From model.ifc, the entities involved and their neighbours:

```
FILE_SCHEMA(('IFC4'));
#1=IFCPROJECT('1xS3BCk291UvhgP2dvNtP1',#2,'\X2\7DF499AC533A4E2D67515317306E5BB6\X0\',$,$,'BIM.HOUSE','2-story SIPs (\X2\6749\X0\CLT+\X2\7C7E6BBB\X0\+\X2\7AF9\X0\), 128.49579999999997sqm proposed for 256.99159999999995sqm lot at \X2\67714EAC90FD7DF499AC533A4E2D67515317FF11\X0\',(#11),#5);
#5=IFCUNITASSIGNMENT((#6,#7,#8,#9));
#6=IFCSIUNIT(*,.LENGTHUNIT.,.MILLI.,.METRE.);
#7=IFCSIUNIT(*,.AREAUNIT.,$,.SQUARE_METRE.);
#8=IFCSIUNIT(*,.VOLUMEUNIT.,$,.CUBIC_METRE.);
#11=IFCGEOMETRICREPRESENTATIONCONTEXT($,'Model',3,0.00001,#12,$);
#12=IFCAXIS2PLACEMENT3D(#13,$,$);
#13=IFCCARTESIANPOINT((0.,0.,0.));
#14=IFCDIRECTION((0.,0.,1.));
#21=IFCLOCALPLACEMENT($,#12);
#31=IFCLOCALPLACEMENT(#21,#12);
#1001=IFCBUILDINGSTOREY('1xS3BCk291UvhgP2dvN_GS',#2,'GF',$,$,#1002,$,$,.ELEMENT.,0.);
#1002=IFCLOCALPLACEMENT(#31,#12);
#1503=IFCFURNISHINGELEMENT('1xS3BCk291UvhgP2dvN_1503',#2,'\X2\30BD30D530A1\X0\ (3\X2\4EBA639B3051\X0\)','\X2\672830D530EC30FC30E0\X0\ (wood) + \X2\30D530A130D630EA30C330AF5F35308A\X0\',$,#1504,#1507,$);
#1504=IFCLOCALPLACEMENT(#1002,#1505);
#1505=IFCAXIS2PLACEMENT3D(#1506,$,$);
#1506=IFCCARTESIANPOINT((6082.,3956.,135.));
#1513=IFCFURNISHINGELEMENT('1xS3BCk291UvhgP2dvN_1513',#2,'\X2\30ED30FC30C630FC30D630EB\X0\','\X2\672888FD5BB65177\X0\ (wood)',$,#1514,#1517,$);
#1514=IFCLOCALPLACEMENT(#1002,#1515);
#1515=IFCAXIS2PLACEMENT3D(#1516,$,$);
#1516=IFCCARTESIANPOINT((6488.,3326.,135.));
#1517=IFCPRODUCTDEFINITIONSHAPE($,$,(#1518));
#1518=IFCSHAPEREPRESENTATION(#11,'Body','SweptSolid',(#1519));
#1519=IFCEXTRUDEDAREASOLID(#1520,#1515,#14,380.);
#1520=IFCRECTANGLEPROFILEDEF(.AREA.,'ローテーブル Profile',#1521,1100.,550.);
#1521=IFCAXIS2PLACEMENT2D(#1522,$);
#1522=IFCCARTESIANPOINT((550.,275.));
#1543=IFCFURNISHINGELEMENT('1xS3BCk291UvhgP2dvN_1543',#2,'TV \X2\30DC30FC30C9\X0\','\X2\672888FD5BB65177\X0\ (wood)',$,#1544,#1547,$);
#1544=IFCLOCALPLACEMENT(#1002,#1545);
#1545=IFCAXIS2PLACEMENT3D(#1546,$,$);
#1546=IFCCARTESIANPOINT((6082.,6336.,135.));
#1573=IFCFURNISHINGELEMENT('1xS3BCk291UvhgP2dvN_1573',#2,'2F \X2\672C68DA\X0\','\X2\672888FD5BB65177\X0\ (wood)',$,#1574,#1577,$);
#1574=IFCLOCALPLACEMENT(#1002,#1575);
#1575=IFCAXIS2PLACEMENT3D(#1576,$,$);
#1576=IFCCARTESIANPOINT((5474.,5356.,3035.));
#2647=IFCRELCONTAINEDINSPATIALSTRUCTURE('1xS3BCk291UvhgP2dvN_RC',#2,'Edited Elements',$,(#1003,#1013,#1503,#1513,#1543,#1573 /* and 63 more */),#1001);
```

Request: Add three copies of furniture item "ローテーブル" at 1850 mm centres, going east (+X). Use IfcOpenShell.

```python
import numpy as np
import ifcopenshell
import ifcopenshell.api.geometry
import ifcopenshell.api.root
import ifcopenshell.util.element
import ifcopenshell.util.placement

model = ifcopenshell.open("model.ifc")


def reuse_history(source, copy):
    """copy_class also copies each property set's owner history, people and application; keep the originals."""
    for rel in copy.IsDefinedBy:
        if rel.is_a("IfcRelDefinesByProperties") and (history := rel.RelatingPropertyDefinition.OwnerHistory):
            rel.RelatingPropertyDefinition.OwnerHistory = source.OwnerHistory
            ifcopenshell.util.element.remove_deep2(model, history)


source = model.by_id(1513)
base = ifcopenshell.util.placement.get_local_placement(source.ObjectPlacement)
step = np.array([1.0, 0.0, 0.0]) * 1850.0

for i in range(1, 4):
    copy = ifcopenshell.api.root.copy_class(model, product=source)
    copy.Representation = ifcopenshell.util.element.copy_deep(
        model, source.Representation, exclude=["IfcGeometricRepresentationContext", "IfcRepresentationMap"]
    )
    reuse_history(source, copy)
    matrix = base.copy()
    matrix[:3, 3] += i * step
    print("added at", matrix[:3, 3].round(3) + 0.0)
    ifcopenshell.api.geometry.edit_object_placement(model, product=copy, matrix=matrix, is_si=False)

model.write("model_updated.ifc")
```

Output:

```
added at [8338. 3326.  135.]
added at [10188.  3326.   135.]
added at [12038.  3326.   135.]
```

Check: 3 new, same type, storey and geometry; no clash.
